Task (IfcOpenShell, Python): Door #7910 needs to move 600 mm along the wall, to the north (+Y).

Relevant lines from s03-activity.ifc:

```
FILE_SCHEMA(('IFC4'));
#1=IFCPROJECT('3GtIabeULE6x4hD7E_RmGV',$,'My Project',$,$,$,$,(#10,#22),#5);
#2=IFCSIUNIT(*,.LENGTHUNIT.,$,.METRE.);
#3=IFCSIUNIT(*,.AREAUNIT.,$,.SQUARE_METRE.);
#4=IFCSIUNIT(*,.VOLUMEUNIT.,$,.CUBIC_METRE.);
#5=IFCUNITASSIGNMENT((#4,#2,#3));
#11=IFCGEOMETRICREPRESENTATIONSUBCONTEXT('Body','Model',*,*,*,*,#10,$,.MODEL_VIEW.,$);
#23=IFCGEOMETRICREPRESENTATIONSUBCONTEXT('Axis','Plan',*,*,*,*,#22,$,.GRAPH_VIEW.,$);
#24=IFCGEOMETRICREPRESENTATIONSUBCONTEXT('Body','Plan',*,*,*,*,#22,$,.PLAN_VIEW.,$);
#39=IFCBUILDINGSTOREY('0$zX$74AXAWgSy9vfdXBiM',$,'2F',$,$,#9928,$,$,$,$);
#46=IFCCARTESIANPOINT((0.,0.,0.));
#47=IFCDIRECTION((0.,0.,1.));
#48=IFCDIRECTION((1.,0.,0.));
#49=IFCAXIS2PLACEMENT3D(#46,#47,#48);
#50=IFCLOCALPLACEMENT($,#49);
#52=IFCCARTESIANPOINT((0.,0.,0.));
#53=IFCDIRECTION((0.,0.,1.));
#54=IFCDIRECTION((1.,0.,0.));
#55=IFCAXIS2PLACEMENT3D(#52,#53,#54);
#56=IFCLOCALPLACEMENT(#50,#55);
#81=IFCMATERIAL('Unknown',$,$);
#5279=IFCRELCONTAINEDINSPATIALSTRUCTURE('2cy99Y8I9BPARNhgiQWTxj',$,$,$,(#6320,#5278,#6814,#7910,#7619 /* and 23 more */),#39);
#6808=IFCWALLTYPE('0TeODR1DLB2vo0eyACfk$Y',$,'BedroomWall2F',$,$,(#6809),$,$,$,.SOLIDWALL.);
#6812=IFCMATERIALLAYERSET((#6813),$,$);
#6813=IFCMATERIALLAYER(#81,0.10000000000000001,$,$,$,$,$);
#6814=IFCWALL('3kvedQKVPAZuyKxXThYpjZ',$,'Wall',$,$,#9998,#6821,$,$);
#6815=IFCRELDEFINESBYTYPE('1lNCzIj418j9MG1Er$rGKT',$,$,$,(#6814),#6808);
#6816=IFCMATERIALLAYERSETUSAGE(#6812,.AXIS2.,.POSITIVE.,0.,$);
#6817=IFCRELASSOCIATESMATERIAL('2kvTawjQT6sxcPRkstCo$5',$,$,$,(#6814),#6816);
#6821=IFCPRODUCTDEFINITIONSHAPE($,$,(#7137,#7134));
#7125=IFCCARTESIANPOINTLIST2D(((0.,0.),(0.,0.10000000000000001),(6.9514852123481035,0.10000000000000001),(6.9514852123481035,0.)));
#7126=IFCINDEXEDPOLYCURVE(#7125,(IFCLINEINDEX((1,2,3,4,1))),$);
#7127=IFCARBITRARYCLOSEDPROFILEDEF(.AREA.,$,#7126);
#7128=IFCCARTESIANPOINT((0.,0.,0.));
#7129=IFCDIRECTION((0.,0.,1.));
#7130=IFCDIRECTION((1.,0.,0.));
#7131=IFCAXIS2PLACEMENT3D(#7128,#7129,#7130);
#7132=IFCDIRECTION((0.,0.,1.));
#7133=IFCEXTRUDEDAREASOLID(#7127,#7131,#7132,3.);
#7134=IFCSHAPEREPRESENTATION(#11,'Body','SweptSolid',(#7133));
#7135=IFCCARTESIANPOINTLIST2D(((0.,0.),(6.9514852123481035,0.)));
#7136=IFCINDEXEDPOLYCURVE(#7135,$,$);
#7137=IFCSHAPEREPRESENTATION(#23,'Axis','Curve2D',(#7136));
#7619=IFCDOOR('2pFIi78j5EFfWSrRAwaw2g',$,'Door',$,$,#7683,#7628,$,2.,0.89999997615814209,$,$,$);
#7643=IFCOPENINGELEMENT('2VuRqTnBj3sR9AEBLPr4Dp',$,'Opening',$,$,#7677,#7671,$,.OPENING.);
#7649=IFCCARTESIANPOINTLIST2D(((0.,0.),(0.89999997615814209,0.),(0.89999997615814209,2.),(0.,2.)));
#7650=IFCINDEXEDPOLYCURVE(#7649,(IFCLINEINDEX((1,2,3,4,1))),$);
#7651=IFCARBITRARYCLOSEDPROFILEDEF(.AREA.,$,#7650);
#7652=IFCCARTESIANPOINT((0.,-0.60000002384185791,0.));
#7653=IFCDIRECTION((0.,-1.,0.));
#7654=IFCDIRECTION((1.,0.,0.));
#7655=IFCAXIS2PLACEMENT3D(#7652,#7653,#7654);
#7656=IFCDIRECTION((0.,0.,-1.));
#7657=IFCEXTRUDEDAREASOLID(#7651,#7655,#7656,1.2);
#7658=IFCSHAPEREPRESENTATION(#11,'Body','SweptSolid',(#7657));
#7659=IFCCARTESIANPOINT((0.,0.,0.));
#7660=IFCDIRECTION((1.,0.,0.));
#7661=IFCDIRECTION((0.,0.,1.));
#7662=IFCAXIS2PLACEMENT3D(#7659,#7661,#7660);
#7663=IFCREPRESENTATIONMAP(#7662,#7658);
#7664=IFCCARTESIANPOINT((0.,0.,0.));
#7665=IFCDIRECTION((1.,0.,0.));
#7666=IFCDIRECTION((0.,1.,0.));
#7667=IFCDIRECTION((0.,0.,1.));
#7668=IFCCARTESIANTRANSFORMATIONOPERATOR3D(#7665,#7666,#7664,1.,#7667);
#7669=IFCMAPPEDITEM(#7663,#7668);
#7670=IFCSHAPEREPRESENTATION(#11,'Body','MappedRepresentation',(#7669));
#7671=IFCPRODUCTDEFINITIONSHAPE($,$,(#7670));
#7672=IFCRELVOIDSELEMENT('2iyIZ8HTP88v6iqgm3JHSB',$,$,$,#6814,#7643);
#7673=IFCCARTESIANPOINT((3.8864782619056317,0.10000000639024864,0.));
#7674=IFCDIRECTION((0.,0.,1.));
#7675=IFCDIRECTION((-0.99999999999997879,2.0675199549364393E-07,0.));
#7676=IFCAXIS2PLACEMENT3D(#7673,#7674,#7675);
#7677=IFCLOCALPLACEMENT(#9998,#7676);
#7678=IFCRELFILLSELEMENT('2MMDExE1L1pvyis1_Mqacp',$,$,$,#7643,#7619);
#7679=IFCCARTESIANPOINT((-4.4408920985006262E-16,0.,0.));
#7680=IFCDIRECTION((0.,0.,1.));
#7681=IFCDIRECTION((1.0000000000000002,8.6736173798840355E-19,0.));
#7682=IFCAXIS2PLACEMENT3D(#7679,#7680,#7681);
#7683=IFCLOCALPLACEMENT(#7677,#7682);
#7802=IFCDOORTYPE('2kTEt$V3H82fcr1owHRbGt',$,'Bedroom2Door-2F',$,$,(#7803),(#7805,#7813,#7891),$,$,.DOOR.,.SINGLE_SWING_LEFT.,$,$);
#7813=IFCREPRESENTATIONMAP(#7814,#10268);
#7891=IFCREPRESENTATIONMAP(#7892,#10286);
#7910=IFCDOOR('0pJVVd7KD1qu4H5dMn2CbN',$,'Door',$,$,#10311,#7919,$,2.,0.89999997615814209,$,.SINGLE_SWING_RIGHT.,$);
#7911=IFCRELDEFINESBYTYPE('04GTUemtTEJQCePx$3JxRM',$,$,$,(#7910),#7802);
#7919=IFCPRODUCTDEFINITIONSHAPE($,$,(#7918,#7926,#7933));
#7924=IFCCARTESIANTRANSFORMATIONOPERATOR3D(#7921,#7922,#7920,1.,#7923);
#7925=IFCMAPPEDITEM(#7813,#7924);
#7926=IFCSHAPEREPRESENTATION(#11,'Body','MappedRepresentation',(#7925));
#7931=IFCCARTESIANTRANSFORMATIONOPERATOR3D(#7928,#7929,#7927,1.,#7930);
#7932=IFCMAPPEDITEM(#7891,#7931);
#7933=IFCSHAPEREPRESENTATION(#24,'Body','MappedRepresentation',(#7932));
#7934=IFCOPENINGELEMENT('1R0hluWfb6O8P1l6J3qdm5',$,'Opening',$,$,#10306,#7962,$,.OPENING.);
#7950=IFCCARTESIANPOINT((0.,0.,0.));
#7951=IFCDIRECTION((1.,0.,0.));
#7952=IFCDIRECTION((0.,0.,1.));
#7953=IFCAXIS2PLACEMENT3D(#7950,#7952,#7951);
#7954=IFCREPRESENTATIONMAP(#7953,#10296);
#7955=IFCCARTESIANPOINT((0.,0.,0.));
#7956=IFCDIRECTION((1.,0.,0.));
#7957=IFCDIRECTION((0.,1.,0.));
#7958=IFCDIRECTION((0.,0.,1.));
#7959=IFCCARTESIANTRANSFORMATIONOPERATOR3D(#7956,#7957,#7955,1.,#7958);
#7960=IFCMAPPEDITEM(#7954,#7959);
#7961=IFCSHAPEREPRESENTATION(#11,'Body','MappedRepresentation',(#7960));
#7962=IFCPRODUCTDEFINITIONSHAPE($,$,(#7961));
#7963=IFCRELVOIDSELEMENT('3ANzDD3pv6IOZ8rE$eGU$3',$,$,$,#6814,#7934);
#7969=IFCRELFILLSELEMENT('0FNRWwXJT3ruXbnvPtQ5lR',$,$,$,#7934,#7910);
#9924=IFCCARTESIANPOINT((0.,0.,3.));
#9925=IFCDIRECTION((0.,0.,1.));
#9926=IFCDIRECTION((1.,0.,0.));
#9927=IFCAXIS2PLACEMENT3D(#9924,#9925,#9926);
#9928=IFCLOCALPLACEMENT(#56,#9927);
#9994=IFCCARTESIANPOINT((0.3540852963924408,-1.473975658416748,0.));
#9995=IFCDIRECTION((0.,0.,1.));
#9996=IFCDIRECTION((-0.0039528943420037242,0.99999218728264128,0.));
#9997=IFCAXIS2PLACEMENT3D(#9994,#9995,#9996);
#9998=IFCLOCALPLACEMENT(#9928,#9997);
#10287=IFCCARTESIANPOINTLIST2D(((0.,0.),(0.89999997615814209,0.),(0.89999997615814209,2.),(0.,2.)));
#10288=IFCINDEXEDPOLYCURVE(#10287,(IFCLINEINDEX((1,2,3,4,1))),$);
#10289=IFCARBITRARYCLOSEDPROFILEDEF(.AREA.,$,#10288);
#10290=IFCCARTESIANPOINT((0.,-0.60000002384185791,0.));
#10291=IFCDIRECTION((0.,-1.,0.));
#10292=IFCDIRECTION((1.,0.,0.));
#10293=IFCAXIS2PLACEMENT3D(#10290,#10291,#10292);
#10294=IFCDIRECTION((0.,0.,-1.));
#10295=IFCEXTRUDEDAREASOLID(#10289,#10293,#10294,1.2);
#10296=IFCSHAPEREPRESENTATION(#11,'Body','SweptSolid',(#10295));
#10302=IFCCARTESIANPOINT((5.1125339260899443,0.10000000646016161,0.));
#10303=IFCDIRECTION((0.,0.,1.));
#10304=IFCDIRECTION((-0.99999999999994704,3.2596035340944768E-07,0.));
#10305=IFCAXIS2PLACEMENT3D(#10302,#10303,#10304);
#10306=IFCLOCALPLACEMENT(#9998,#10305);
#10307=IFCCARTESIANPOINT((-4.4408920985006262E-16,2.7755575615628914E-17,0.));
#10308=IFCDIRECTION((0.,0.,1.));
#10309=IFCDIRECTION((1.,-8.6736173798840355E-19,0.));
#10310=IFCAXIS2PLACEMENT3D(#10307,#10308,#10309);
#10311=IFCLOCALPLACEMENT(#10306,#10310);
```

```python
import ifcopenshell
import ifcopenshell.api.geometry
import ifcopenshell.util.placement

model = ifcopenshell.open("s03-activity.ifc")

door = model.by_guid("0pJVVd7KD1qu4H5dMn2CbN")
opening = door.FillsVoids[0].RelatingOpeningElement
wall = opening.VoidsElements[0].RelatingBuildingElement

wall_matrix = ifcopenshell.util.placement.get_local_placement(wall.ObjectPlacement)
shift = wall_matrix[:3, 0] * 0.6
before = ifcopenshell.util.placement.get_local_placement(door.ObjectPlacement)[:3, 3].copy()

# The door is placed relative to its opening, so it follows when the opening moves.
matrix = ifcopenshell.util.placement.get_local_placement(opening.ObjectPlacement)
matrix[:3, 3] += shift
ifcopenshell.api.geometry.edit_object_placement(
    model, product=opening, matrix=matrix, is_si=False, should_transform_children=True
)

after = ifcopenshell.util.placement.get_local_placement(door.ObjectPlacement)[:3, 3]
print("door moved by", (after - before).round(3) + 0.0)

model.write("s03-activity_edited.ifc")
```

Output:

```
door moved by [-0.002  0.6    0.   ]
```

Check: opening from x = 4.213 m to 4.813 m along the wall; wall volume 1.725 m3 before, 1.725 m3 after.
